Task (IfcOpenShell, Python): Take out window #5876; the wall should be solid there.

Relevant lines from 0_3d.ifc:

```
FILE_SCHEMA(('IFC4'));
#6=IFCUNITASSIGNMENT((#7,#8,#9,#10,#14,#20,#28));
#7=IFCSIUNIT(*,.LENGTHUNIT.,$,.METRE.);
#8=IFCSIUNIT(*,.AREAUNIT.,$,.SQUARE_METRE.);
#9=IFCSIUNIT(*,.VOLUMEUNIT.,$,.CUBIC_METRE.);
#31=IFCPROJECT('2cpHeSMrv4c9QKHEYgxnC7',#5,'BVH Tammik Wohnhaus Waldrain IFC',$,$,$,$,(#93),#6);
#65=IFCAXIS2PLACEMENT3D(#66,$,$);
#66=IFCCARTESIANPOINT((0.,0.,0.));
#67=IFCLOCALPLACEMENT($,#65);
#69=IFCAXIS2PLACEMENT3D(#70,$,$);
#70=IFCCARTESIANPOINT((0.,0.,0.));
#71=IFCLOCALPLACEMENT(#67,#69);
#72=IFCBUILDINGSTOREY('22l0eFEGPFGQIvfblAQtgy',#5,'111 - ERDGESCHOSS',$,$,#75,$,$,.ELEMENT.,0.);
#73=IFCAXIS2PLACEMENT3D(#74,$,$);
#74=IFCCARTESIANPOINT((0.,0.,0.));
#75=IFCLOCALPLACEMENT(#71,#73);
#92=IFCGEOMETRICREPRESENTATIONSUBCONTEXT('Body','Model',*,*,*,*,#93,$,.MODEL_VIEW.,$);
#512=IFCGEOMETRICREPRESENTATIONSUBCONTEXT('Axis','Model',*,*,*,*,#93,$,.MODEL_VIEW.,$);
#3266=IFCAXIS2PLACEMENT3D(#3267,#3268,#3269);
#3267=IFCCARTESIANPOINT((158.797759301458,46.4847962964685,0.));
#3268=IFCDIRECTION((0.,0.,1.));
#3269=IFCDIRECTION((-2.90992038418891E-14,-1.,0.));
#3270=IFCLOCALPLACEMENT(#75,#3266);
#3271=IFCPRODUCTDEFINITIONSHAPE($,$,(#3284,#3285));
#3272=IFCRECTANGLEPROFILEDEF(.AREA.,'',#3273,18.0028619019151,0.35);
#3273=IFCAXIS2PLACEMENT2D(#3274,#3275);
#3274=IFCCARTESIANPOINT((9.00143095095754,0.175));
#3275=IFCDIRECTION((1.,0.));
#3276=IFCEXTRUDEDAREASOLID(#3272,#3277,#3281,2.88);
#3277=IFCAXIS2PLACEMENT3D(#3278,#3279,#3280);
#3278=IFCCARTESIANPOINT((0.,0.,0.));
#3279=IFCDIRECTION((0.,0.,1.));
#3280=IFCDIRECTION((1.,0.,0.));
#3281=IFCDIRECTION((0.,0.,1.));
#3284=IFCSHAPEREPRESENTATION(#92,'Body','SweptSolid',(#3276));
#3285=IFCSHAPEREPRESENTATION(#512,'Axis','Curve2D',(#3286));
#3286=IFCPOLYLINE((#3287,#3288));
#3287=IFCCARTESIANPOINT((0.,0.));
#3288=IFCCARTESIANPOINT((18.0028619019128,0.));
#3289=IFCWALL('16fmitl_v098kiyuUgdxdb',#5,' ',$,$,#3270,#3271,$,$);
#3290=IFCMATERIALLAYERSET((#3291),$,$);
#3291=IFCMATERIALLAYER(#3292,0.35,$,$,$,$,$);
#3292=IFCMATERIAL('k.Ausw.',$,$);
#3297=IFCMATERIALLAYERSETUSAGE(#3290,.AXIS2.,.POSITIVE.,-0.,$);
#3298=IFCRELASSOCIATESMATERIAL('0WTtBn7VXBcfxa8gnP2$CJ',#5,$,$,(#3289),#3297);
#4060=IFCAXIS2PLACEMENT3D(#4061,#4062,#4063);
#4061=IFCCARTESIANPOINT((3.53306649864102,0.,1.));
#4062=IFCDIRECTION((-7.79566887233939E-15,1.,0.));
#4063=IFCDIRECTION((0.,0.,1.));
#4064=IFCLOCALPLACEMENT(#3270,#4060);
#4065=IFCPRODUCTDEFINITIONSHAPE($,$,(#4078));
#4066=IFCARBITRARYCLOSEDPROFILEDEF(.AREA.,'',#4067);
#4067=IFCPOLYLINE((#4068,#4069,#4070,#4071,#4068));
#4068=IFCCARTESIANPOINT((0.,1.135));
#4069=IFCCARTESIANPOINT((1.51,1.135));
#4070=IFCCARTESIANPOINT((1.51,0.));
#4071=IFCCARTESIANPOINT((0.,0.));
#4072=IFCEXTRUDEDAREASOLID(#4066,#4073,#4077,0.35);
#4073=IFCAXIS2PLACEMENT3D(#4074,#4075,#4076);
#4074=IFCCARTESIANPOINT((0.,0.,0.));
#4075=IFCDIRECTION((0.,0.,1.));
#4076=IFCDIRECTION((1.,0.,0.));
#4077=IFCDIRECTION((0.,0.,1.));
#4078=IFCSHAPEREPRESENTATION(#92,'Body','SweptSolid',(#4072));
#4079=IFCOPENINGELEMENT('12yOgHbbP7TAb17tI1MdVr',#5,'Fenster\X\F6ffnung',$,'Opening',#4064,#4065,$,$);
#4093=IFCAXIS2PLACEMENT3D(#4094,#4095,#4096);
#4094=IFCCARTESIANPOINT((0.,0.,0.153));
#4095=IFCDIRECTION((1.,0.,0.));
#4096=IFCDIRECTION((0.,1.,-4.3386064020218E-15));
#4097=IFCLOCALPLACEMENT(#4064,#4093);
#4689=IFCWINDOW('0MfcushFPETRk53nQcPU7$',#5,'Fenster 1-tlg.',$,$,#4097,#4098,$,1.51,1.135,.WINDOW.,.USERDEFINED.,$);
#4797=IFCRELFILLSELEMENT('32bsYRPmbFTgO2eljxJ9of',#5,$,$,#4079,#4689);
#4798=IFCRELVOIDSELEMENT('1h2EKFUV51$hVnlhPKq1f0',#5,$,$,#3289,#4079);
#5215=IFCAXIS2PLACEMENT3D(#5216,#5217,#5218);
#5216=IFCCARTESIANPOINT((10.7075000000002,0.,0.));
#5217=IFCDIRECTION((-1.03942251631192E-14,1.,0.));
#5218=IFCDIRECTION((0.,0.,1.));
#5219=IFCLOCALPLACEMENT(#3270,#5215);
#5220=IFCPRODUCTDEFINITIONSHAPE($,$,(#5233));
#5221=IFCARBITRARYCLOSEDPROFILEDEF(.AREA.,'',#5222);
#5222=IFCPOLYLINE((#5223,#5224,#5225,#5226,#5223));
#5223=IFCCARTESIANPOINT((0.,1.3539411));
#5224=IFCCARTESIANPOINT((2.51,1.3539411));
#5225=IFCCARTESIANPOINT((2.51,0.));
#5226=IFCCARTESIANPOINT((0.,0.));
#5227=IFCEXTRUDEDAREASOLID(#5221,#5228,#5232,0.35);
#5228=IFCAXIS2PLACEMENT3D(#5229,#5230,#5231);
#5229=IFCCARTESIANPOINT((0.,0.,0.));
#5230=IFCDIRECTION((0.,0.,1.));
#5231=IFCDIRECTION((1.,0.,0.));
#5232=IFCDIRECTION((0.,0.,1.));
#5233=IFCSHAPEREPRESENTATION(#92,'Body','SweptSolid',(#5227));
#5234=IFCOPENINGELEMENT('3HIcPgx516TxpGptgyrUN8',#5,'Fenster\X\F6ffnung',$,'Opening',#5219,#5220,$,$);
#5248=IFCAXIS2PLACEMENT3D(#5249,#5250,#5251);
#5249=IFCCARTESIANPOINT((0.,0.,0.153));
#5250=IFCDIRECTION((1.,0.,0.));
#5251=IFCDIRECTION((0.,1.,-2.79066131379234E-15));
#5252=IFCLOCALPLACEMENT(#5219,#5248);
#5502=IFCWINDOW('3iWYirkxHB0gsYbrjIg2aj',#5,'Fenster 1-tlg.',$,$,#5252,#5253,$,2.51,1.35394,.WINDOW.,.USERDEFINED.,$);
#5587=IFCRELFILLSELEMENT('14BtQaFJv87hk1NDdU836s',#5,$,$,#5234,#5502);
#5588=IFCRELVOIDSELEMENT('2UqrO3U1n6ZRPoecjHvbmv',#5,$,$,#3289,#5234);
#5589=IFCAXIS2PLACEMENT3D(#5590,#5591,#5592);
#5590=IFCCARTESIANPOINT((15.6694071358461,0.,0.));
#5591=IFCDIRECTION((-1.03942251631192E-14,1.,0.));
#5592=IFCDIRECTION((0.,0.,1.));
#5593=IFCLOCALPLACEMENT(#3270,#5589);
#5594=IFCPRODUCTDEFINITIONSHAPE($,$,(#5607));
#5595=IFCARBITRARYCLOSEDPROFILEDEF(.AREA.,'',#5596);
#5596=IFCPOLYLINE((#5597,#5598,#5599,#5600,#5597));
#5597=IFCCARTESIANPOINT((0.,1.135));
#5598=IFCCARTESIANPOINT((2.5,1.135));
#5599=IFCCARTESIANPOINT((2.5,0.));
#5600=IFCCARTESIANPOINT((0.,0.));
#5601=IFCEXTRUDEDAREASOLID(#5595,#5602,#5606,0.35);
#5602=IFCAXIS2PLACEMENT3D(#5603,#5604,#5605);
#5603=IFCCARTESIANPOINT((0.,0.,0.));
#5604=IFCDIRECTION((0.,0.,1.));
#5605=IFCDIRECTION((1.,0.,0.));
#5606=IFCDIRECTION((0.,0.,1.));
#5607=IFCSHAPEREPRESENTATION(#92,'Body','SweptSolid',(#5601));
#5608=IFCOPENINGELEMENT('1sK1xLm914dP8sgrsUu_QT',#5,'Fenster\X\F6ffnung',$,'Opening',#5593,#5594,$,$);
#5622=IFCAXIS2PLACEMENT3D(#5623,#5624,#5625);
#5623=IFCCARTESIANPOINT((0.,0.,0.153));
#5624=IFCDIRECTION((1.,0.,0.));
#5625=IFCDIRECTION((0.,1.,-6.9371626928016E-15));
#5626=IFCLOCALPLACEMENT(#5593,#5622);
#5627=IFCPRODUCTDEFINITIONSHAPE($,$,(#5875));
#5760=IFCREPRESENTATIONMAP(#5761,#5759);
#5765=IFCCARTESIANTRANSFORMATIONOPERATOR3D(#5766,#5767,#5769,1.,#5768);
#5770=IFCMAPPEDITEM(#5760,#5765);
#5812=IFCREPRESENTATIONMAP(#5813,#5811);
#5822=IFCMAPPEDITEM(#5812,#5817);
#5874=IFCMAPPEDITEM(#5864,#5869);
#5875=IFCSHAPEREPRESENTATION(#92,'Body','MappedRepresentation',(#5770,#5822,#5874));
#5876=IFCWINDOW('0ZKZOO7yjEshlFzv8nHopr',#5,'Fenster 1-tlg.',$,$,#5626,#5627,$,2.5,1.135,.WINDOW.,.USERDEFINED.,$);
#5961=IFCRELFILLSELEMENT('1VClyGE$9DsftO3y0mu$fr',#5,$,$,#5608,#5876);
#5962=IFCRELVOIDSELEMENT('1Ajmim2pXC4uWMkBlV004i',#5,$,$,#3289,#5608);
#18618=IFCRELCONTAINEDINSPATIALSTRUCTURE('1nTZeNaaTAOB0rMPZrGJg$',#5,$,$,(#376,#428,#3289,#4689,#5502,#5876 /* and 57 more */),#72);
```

```python
import ifcopenshell
import ifcopenshell.api.feature
import ifcopenshell.api.root
import ifcopenshell.geom
import ifcopenshell.util.shape

model = ifcopenshell.open("0_3d.ifc")
settings = ifcopenshell.geom.settings()


def volume(element):
    """Net volume in cubic metres, openings subtracted."""
    shape = ifcopenshell.geom.create_shape(settings, element)
    return ifcopenshell.util.shape.get_volume(shape.geometry)


window = model.by_guid("0ZKZOO7yjEshlFzv8nHopr")
opening = window.FillsVoids[0].RelatingOpeningElement
wall = opening.VoidsElements[0].RelatingBuildingElement
before = volume(wall)

ifcopenshell.api.root.remove_product(model, product=window)
ifcopenshell.api.feature.remove_feature(model, feature=opening)

after = volume(wall)

print(f"wall volume {before:.3f} -> {after:.3f} m3")

model.write("0_3d_v2.ifc")
```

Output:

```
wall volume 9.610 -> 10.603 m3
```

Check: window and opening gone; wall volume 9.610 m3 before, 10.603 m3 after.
